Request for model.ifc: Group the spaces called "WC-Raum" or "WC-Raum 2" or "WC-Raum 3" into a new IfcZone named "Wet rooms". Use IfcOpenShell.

First a look at what the model holds.

```python
import ifcopenshell

model = ifcopenshell.open("model.ifc")
print(model.schema)
seen = {}
for space in model.by_type("IfcSpace"):
    seen[space.Name] = seen.get(space.Name, 0) + 1
for name, count in sorted(seen.items(), key=str):
    print(count, "x", name)
print("zones:", [z.Name for z in model.by_type("IfcZone")][:20])
```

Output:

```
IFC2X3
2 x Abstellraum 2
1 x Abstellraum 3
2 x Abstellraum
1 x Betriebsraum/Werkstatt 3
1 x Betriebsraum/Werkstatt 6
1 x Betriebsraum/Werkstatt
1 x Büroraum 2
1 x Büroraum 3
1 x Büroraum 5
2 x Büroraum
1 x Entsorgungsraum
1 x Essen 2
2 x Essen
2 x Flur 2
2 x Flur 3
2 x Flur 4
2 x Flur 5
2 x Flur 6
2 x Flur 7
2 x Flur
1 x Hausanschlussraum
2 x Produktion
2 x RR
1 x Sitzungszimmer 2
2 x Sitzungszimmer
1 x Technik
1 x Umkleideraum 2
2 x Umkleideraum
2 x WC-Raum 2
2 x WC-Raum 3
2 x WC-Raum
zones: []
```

```python
import ifcopenshell
import ifcopenshell.api.group
import ifcopenshell.api.root

model = ifcopenshell.open("model.ifc")

names = {"WC-Raum", "WC-Raum 2", "WC-Raum 3"}
spaces = [s for s in model.by_type("IfcSpace") if s.Name in names]

zone = ifcopenshell.api.root.create_entity(model, ifc_class="IfcZone", name="Wet rooms")
ifcopenshell.api.group.assign_group(model, products=spaces, group=zone)
print(len(spaces), "spaces in", zone.Name)

model.write("model_edited.ifc")
```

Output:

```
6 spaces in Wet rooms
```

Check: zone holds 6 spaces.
